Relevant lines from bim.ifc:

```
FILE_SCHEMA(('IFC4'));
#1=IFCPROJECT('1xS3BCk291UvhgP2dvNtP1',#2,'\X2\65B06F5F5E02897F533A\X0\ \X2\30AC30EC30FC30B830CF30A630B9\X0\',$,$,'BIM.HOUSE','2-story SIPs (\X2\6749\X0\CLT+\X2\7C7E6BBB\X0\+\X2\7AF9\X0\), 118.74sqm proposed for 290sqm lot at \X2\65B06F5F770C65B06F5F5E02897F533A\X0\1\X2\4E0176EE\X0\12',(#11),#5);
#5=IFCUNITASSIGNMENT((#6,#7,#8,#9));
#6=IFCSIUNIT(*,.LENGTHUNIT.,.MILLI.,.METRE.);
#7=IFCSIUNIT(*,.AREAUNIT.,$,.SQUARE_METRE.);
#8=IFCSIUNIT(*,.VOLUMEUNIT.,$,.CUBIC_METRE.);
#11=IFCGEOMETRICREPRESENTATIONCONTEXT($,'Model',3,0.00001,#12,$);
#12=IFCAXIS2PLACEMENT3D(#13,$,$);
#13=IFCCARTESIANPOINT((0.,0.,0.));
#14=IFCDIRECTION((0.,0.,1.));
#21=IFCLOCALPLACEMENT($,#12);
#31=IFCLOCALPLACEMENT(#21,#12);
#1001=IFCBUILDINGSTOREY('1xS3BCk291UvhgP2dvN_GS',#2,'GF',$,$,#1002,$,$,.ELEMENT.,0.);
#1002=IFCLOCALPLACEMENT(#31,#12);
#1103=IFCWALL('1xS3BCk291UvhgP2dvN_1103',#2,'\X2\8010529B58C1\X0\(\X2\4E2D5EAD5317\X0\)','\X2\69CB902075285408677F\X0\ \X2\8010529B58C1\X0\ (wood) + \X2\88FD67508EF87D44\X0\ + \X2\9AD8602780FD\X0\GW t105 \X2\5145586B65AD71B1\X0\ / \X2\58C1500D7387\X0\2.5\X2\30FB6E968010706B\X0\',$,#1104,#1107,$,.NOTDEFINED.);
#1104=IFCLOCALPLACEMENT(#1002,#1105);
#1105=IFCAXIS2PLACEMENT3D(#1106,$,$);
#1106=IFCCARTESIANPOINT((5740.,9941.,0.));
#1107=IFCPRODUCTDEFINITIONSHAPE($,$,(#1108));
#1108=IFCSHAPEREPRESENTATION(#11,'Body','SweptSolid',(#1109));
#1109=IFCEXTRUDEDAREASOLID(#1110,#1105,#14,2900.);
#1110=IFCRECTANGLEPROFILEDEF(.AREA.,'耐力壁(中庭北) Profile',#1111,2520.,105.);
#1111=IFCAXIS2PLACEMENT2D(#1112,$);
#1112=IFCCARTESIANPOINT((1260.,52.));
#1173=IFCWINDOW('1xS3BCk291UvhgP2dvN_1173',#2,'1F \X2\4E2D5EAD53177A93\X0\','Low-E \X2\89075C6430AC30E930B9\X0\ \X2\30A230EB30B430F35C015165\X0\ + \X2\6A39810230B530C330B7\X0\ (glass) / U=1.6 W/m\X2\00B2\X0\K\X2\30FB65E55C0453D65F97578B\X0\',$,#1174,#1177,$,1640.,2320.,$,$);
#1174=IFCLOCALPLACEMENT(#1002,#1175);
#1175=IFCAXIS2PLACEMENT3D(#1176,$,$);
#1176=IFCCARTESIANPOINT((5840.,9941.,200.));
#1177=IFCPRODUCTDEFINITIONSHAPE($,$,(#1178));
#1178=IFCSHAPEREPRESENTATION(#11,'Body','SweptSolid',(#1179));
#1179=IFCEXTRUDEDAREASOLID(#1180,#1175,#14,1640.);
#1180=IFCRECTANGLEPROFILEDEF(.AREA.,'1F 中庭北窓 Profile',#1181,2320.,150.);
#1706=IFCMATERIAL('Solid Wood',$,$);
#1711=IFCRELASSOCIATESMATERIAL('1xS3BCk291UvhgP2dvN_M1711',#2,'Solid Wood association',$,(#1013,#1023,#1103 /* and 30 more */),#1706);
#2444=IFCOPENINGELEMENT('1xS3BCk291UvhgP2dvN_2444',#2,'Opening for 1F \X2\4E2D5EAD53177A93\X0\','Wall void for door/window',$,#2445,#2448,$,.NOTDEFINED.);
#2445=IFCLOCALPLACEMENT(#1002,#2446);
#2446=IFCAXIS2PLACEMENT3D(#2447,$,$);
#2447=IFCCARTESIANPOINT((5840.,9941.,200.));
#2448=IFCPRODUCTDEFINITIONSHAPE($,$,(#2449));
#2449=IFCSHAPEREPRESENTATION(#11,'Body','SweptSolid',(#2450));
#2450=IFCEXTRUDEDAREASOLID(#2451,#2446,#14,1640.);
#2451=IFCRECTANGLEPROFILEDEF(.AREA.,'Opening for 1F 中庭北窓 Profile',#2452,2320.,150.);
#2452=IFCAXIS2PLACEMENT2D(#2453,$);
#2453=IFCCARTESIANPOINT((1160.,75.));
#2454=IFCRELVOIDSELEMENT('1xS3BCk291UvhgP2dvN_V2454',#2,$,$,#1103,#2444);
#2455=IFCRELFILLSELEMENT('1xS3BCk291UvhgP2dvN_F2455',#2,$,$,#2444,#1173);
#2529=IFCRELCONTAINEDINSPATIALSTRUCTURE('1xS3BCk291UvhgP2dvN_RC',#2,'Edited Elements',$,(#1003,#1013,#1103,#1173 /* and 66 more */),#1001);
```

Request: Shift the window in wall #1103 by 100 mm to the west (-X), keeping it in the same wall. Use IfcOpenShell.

```python
import ifcopenshell
import ifcopenshell.api.geometry
import ifcopenshell.util.placement
import ifcopenshell.util.unit

model = ifcopenshell.open("bim.ifc")
unit_scale = ifcopenshell.util.unit.calculate_unit_scale(model)

window = model.by_guid("1xS3BCk291UvhgP2dvN_1173")
opening = window.FillsVoids[0].RelatingOpeningElement
wall = opening.VoidsElements[0].RelatingBuildingElement

wall_matrix = ifcopenshell.util.placement.get_local_placement(wall.ObjectPlacement)
shift = wall_matrix[:3, 0] * -0.1 / unit_scale
before = ifcopenshell.util.placement.get_local_placement(window.ObjectPlacement)[:3, 3].copy()

# The window is not placed relative to its opening, so move both.
for product in (opening, window):
    matrix = ifcopenshell.util.placement.get_local_placement(product.ObjectPlacement)
    matrix[:3, 3] += shift
    ifcopenshell.api.geometry.edit_object_placement(model, product=product, matrix=matrix, is_si=False)

after = ifcopenshell.util.placement.get_local_placement(window.ObjectPlacement)[:3, 3]
print("window moved by", (after - before).round(3) + 0.0)

model.write("bim_rev.ifc")
```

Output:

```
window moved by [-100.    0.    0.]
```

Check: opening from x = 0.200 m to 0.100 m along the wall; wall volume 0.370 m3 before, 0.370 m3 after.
